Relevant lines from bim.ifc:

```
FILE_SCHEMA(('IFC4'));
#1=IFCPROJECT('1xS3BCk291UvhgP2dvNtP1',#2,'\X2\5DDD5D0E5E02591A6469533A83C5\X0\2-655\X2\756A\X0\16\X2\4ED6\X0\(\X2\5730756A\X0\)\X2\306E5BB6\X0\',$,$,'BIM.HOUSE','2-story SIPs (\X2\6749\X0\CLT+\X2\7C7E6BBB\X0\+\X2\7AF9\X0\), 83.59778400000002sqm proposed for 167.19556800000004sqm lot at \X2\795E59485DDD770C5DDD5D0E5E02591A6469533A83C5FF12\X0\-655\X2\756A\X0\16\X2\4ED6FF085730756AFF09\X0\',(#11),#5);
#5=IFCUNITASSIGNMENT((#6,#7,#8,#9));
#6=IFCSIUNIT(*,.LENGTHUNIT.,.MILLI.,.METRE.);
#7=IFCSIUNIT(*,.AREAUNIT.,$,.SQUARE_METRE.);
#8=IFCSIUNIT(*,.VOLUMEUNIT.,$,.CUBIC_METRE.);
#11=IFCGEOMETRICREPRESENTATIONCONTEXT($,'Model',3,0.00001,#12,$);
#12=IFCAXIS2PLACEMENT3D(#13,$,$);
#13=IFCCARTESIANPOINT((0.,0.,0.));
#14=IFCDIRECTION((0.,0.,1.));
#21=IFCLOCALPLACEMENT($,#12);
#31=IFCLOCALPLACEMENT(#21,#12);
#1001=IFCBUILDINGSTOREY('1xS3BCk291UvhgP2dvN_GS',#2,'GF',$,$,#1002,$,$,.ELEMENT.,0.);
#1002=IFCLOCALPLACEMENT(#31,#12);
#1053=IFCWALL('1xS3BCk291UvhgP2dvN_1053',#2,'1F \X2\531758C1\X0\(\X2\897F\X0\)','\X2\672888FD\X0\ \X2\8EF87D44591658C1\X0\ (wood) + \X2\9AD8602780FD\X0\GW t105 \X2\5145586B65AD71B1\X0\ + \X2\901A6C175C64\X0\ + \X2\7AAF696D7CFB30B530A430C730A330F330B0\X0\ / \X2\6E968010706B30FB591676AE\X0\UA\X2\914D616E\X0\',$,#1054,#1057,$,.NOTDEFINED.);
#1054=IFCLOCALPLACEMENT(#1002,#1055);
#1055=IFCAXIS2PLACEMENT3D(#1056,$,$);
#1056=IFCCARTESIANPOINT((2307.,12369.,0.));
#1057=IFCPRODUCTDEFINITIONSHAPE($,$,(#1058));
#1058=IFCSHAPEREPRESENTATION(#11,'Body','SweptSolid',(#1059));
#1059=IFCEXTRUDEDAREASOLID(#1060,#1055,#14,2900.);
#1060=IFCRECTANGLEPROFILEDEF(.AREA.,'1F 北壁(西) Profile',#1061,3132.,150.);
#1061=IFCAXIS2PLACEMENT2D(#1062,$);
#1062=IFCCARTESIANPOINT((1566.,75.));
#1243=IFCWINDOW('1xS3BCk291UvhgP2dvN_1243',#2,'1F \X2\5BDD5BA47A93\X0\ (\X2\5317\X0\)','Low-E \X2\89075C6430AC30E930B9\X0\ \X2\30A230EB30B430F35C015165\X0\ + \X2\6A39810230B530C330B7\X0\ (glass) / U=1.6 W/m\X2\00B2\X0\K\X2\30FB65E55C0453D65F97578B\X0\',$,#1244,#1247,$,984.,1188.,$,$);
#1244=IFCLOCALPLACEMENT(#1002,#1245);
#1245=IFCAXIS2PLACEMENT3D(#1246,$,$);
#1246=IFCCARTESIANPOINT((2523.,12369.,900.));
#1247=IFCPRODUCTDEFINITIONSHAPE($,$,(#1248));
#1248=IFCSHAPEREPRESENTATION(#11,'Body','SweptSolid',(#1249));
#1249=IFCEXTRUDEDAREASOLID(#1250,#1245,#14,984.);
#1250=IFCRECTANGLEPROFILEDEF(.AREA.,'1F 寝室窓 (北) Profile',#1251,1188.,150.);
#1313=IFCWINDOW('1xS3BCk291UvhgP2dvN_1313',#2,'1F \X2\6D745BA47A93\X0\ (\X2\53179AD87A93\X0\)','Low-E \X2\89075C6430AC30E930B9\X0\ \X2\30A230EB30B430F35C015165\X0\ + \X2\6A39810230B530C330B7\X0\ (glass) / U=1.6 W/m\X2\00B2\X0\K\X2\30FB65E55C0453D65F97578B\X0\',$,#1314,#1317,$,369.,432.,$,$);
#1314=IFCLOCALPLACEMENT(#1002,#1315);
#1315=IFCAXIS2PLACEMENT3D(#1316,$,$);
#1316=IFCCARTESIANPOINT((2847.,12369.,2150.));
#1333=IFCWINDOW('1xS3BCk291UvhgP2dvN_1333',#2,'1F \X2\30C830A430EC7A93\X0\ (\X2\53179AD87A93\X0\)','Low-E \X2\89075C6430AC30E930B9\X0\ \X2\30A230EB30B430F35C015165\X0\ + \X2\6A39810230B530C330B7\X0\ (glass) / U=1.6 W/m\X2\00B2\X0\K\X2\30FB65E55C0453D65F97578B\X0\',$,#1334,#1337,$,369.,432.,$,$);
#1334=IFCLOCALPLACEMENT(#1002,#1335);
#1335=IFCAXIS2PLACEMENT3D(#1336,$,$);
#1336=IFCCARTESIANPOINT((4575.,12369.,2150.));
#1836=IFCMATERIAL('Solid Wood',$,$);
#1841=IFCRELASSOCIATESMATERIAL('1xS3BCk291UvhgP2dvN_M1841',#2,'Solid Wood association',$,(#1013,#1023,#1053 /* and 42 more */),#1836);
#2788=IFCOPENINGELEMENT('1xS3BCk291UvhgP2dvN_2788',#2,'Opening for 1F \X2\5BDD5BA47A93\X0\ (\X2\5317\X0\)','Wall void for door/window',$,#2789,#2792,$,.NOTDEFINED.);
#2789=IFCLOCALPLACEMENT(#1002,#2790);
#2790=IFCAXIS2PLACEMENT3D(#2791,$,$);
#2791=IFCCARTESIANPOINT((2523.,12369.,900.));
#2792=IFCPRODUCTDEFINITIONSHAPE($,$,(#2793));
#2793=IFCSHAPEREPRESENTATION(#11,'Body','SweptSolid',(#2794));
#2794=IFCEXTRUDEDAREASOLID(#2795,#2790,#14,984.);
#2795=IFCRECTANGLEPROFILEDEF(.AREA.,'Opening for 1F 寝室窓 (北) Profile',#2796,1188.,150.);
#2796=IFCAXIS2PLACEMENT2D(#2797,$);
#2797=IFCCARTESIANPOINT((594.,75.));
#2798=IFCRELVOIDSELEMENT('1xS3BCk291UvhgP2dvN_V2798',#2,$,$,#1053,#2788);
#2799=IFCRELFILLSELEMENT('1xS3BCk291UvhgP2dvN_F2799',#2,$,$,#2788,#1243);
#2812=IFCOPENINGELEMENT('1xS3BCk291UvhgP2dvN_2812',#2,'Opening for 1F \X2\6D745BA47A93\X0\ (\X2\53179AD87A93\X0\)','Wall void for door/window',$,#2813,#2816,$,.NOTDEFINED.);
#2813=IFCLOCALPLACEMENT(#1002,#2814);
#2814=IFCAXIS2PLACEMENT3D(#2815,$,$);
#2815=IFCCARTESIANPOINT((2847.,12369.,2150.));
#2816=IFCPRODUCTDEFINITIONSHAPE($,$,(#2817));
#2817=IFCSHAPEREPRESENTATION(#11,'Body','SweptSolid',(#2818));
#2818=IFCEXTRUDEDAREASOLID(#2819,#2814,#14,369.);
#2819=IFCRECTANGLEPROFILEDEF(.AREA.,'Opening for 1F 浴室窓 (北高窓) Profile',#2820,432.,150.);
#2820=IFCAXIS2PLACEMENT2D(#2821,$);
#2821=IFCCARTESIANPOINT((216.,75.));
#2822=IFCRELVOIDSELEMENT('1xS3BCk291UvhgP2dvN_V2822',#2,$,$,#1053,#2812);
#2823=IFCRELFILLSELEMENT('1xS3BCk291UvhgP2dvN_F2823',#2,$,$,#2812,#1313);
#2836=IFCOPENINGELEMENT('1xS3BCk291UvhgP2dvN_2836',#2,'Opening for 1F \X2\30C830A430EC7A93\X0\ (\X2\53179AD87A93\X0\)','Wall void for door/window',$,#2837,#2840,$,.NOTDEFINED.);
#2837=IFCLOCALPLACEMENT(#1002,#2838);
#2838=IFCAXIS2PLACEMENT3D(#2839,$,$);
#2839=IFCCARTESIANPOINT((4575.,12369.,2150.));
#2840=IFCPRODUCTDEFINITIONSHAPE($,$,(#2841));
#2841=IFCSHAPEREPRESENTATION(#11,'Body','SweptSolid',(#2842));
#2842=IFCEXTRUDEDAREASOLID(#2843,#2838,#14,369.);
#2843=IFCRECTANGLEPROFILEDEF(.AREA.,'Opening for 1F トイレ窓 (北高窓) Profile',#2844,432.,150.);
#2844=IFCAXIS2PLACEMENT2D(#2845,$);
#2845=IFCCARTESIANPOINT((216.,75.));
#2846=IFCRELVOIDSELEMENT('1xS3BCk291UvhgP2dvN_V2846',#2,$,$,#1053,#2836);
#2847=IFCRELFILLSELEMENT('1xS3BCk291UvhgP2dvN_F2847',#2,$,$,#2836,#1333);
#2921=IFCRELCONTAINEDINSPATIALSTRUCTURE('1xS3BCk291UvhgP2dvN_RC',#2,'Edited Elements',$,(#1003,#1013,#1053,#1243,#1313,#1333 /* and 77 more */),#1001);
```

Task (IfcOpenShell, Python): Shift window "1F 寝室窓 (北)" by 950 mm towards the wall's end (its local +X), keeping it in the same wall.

```python
import ifcopenshell
import ifcopenshell.api.geometry
import ifcopenshell.util.placement
import ifcopenshell.util.unit

model = ifcopenshell.open("bim.ifc")
unit_scale = ifcopenshell.util.unit.calculate_unit_scale(model)

window = model.by_id(1243)
opening = window.FillsVoids[0].RelatingOpeningElement
wall = opening.VoidsElements[0].RelatingBuildingElement

wall_matrix = ifcopenshell.util.placement.get_local_placement(wall.ObjectPlacement)
shift = wall_matrix[:3, 0] * 0.95 / unit_scale
before = ifcopenshell.util.placement.get_local_placement(window.ObjectPlacement)[:3, 3].copy()

# The window is not placed relative to its opening, so move both.
for product in (opening, window):
    matrix = ifcopenshell.util.placement.get_local_placement(product.ObjectPlacement)
    matrix[:3, 3] += shift
    ifcopenshell.api.geometry.edit_object_placement(model, product=product, matrix=matrix, is_si=False)

after = ifcopenshell.util.placement.get_local_placement(window.ObjectPlacement)[:3, 3]
print("window moved by", (after - before).round(3) + 0.0)

model.write("bim_edited.ifc")
```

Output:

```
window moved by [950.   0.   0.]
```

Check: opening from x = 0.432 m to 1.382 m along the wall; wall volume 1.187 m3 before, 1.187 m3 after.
